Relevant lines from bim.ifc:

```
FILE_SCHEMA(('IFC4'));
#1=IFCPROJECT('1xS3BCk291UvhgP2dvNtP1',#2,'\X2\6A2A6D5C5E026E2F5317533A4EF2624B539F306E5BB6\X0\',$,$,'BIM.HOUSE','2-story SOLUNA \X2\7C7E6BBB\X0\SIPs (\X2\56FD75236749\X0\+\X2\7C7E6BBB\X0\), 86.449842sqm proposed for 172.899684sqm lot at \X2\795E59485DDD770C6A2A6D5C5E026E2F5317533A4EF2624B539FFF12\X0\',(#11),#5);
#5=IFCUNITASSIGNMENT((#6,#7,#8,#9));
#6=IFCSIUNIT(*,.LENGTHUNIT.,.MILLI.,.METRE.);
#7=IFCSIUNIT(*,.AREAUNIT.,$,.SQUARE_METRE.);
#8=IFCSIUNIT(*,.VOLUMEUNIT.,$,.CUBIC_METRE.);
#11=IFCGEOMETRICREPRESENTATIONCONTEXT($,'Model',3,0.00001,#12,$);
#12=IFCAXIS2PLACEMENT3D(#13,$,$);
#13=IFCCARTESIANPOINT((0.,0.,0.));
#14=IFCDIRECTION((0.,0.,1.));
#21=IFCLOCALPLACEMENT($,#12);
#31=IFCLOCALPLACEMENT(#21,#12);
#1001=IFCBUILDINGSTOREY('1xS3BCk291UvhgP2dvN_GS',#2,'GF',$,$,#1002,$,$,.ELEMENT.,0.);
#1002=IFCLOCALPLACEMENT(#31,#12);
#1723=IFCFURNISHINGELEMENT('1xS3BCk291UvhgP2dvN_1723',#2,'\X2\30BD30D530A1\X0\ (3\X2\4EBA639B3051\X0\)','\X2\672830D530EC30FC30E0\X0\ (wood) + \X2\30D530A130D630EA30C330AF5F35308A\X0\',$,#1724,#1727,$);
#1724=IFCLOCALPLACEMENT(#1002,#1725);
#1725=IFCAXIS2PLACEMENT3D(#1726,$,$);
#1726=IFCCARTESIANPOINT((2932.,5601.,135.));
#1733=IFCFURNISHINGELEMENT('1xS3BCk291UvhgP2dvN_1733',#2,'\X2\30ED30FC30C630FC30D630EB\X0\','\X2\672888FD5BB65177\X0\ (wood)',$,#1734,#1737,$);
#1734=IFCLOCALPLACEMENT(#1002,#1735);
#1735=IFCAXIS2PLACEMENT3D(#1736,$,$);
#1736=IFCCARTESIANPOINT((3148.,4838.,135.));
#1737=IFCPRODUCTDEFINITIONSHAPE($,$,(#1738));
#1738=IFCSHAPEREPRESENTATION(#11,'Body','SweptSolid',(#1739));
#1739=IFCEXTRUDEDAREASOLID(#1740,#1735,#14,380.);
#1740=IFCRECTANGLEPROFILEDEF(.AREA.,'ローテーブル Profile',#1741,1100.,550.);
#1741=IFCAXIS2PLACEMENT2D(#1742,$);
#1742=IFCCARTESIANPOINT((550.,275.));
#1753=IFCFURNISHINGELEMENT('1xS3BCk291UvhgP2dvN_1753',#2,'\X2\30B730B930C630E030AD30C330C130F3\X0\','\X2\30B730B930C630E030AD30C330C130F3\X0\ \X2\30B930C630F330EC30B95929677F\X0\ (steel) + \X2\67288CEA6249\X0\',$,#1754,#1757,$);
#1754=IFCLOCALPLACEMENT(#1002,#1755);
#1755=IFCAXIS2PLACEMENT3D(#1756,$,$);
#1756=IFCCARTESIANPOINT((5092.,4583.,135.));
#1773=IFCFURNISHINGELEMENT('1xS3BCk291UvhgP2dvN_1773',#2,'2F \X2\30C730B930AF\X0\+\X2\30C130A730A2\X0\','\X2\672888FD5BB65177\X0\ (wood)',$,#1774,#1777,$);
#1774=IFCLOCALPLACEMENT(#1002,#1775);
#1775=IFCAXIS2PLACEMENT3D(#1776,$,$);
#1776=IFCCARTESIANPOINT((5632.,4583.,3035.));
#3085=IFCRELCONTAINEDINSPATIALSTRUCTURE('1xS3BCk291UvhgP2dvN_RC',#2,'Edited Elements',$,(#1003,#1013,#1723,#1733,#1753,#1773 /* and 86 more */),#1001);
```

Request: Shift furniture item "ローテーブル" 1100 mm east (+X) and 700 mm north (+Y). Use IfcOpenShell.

```python
import ifcopenshell
import ifcopenshell.api.geometry
import ifcopenshell.util.placement

model = ifcopenshell.open("bim.ifc")

item = model.by_guid("1xS3BCk291UvhgP2dvN_1733")
matrix = ifcopenshell.util.placement.get_local_placement(item.ObjectPlacement)
matrix[0, 3] += 1100.0
matrix[1, 3] += 700.0
ifcopenshell.api.geometry.edit_object_placement(model, product=item, matrix=matrix, is_si=False)

print(ifcopenshell.util.placement.get_local_placement(item.ObjectPlacement).round(3) + 0.0)

model.write("bim-out.ifc")
```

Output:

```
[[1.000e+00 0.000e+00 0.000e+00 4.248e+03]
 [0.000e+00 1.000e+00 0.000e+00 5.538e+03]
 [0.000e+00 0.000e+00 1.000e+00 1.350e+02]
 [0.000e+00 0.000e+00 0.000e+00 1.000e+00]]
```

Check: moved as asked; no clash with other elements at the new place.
